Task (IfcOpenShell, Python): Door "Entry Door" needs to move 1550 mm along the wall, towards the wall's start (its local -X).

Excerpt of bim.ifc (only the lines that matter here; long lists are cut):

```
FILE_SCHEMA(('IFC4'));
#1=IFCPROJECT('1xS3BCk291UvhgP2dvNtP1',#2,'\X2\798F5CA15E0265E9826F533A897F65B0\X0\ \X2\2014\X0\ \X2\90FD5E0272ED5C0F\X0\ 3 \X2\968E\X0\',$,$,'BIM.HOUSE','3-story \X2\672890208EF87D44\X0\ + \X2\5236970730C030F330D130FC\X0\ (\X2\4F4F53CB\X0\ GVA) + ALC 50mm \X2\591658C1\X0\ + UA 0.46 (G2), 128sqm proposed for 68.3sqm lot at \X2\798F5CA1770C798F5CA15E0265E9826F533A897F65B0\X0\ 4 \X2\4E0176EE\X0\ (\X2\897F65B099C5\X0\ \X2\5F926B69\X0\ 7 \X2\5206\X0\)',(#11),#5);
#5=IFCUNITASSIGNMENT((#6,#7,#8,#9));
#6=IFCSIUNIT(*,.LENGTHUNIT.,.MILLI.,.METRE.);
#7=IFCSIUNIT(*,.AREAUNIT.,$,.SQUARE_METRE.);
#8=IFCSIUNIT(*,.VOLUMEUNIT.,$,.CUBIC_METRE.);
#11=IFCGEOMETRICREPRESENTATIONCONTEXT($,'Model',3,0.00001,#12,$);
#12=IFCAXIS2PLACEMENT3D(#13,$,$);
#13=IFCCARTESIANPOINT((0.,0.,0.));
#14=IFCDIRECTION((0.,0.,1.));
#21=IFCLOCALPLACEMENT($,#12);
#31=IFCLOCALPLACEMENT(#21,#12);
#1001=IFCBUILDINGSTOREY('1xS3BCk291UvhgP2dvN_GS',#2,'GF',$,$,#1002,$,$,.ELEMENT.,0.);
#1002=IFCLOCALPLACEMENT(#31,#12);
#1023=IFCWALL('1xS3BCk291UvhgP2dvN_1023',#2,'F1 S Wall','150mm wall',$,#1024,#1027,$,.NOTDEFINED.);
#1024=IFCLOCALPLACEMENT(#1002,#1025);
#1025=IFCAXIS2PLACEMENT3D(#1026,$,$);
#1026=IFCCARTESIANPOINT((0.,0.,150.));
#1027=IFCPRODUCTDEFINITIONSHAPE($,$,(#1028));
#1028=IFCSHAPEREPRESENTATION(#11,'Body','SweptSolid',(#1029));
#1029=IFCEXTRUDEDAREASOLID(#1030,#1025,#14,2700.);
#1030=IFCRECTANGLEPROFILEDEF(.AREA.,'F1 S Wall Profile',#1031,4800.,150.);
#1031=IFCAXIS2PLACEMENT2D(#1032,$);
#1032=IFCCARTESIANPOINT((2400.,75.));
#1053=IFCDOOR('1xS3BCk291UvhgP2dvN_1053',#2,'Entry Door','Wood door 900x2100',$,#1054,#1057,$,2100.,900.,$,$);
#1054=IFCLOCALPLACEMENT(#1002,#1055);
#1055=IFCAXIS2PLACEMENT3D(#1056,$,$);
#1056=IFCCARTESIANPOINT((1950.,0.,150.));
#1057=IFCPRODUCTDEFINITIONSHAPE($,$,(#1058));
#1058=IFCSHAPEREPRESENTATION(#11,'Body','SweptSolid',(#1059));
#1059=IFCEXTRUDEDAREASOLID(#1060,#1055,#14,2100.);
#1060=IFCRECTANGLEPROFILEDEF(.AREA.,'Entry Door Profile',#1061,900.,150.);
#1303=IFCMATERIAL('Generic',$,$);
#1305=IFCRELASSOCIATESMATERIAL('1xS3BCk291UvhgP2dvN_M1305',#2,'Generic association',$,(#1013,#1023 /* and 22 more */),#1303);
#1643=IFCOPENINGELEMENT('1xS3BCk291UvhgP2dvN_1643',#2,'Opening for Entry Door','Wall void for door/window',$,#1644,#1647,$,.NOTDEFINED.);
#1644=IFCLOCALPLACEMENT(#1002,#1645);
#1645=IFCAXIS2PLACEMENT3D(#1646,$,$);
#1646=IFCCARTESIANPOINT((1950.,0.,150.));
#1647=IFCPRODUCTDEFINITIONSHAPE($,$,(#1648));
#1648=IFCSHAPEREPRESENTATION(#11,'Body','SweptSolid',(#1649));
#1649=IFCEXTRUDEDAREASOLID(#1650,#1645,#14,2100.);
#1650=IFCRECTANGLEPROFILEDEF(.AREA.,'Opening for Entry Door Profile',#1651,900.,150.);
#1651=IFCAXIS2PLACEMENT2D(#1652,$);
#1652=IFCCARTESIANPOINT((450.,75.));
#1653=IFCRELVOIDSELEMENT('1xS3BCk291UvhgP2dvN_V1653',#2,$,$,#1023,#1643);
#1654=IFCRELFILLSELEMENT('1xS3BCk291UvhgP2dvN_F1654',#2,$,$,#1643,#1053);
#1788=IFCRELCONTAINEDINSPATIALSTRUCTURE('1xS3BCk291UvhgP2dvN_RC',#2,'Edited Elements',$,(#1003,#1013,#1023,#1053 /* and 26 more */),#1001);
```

```python
import ifcopenshell
import ifcopenshell.api.geometry
import ifcopenshell.util.placement

model = ifcopenshell.open("bim.ifc")

door = model.by_guid("1xS3BCk291UvhgP2dvN_1053")
opening = door.FillsVoids[0].RelatingOpeningElement
wall = opening.VoidsElements[0].RelatingBuildingElement

wall_matrix = ifcopenshell.util.placement.get_local_placement(wall.ObjectPlacement)
shift = wall_matrix[:3, 0] * -1550.0
before = ifcopenshell.util.placement.get_local_placement(door.ObjectPlacement)[:3, 3].copy()

# The door is not placed relative to its opening, so move both.
for product in (opening, door):
    matrix = ifcopenshell.util.placement.get_local_placement(product.ObjectPlacement)
    matrix[:3, 3] += shift
    ifcopenshell.api.geometry.edit_object_placement(model, product=product, matrix=matrix, is_si=False)

after = ifcopenshell.util.placement.get_local_placement(door.ObjectPlacement)[:3, 3]
print("door moved by", (after - before).round(3) + 0.0)

model.write("bim-out.ifc")
```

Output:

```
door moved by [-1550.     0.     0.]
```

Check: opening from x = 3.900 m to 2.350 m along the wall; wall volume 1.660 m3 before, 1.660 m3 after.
